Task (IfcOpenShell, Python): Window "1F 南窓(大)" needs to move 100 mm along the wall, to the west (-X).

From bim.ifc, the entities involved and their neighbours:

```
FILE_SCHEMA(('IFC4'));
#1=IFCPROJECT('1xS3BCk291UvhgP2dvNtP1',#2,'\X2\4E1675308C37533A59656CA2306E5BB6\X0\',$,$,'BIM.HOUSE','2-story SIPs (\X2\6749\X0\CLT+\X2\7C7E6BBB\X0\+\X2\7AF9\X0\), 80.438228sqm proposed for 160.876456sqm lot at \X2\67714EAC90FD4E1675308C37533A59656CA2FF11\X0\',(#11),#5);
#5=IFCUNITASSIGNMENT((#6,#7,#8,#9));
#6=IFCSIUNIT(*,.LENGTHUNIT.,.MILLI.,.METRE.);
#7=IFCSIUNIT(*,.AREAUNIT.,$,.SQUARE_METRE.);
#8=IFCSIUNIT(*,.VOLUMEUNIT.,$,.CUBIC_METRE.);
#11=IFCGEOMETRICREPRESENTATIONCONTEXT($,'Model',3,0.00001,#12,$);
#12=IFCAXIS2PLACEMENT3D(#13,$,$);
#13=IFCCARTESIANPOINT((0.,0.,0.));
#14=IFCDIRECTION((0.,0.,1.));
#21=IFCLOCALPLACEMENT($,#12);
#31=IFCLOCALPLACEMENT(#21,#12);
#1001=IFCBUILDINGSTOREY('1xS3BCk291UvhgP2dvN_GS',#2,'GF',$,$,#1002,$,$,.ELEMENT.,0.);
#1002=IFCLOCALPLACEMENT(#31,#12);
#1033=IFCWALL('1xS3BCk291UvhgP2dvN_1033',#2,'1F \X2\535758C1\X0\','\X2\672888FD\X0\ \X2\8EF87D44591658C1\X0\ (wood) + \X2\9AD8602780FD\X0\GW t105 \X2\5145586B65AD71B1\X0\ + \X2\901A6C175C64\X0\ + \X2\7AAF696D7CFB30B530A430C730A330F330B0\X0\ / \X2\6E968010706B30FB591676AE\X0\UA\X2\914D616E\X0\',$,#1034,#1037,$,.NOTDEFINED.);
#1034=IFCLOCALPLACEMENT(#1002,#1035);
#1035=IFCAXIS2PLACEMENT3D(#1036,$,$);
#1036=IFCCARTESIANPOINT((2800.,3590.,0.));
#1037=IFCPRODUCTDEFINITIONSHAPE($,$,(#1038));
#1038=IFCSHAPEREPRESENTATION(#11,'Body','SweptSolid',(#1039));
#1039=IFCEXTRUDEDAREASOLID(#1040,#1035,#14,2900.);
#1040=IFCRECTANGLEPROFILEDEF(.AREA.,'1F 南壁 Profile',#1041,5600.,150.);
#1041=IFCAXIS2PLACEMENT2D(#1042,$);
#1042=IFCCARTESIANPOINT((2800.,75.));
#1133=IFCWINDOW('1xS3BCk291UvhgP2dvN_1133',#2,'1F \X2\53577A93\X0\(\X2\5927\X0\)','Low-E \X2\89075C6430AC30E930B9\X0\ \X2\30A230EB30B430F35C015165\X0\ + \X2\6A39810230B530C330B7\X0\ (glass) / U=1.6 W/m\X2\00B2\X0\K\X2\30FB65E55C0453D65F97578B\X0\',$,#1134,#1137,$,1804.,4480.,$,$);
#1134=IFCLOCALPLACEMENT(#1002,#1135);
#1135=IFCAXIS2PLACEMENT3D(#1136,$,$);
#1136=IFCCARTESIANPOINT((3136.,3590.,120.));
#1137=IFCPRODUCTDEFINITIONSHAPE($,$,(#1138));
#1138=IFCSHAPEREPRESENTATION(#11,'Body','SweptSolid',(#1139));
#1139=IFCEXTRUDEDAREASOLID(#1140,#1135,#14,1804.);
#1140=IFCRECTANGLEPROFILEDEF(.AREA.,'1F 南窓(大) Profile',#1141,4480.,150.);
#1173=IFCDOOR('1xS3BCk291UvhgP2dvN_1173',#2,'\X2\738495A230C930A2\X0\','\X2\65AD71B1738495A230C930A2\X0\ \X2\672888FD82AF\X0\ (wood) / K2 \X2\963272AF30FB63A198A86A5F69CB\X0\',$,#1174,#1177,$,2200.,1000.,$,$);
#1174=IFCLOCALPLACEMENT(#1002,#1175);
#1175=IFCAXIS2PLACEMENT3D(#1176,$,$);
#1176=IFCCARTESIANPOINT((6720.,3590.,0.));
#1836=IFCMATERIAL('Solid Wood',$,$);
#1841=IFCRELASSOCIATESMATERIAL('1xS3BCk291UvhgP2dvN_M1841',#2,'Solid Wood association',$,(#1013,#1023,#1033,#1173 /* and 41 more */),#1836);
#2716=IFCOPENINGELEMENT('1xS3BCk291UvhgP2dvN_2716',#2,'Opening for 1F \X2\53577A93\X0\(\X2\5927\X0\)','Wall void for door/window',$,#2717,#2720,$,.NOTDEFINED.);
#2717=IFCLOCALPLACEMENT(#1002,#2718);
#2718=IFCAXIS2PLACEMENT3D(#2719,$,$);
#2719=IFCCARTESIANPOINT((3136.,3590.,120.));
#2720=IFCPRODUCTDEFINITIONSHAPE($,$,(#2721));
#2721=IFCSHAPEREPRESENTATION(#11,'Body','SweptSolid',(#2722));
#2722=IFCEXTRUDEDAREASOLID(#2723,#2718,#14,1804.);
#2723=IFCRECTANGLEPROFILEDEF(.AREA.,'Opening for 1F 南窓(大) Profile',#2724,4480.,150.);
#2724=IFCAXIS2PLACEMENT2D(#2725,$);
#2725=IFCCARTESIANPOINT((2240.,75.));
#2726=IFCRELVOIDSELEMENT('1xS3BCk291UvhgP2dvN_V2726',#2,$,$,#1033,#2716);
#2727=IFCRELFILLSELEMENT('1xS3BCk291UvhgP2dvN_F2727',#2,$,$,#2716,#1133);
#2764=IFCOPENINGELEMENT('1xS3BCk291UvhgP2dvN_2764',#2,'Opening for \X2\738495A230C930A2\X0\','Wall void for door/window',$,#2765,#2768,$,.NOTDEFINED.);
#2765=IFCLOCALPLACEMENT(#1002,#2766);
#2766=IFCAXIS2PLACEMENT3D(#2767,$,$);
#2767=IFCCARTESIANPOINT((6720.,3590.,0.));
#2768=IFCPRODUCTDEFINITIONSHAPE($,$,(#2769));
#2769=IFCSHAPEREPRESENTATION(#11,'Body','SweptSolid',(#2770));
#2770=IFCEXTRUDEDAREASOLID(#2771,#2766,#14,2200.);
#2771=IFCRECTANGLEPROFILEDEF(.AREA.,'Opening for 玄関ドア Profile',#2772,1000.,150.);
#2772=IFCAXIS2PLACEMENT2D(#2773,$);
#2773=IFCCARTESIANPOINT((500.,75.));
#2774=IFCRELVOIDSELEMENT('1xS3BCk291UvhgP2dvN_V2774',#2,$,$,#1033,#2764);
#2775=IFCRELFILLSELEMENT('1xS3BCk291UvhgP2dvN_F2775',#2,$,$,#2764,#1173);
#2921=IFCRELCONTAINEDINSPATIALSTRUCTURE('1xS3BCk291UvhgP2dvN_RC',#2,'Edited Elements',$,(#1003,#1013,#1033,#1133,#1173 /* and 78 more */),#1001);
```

```python
import ifcopenshell
import ifcopenshell.api.geometry
import ifcopenshell.util.placement
import ifcopenshell.util.unit

model = ifcopenshell.open("bim.ifc")
unit_scale = ifcopenshell.util.unit.calculate_unit_scale(model)

window = model.by_guid("1xS3BCk291UvhgP2dvN_1133")
opening = window.FillsVoids[0].RelatingOpeningElement
wall = opening.VoidsElements[0].RelatingBuildingElement

wall_matrix = ifcopenshell.util.placement.get_local_placement(wall.ObjectPlacement)
shift = wall_matrix[:3, 0] * -0.1 / unit_scale
before = ifcopenshell.util.placement.get_local_placement(window.ObjectPlacement)[:3, 3].copy()

# The window is not placed relative to its opening, so move both.
for product in (opening, window):
    matrix = ifcopenshell.util.placement.get_local_placement(product.ObjectPlacement)
    matrix[:3, 3] += shift
    ifcopenshell.api.geometry.edit_object_placement(model, product=product, matrix=matrix, is_si=False)

after = ifcopenshell.util.placement.get_local_placement(window.ObjectPlacement)[:3, 3]
print("window moved by", (after - before).round(3) + 0.0)

model.write("bim-out.ifc")
```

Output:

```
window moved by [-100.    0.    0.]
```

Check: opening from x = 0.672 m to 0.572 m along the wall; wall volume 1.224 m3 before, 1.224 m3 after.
